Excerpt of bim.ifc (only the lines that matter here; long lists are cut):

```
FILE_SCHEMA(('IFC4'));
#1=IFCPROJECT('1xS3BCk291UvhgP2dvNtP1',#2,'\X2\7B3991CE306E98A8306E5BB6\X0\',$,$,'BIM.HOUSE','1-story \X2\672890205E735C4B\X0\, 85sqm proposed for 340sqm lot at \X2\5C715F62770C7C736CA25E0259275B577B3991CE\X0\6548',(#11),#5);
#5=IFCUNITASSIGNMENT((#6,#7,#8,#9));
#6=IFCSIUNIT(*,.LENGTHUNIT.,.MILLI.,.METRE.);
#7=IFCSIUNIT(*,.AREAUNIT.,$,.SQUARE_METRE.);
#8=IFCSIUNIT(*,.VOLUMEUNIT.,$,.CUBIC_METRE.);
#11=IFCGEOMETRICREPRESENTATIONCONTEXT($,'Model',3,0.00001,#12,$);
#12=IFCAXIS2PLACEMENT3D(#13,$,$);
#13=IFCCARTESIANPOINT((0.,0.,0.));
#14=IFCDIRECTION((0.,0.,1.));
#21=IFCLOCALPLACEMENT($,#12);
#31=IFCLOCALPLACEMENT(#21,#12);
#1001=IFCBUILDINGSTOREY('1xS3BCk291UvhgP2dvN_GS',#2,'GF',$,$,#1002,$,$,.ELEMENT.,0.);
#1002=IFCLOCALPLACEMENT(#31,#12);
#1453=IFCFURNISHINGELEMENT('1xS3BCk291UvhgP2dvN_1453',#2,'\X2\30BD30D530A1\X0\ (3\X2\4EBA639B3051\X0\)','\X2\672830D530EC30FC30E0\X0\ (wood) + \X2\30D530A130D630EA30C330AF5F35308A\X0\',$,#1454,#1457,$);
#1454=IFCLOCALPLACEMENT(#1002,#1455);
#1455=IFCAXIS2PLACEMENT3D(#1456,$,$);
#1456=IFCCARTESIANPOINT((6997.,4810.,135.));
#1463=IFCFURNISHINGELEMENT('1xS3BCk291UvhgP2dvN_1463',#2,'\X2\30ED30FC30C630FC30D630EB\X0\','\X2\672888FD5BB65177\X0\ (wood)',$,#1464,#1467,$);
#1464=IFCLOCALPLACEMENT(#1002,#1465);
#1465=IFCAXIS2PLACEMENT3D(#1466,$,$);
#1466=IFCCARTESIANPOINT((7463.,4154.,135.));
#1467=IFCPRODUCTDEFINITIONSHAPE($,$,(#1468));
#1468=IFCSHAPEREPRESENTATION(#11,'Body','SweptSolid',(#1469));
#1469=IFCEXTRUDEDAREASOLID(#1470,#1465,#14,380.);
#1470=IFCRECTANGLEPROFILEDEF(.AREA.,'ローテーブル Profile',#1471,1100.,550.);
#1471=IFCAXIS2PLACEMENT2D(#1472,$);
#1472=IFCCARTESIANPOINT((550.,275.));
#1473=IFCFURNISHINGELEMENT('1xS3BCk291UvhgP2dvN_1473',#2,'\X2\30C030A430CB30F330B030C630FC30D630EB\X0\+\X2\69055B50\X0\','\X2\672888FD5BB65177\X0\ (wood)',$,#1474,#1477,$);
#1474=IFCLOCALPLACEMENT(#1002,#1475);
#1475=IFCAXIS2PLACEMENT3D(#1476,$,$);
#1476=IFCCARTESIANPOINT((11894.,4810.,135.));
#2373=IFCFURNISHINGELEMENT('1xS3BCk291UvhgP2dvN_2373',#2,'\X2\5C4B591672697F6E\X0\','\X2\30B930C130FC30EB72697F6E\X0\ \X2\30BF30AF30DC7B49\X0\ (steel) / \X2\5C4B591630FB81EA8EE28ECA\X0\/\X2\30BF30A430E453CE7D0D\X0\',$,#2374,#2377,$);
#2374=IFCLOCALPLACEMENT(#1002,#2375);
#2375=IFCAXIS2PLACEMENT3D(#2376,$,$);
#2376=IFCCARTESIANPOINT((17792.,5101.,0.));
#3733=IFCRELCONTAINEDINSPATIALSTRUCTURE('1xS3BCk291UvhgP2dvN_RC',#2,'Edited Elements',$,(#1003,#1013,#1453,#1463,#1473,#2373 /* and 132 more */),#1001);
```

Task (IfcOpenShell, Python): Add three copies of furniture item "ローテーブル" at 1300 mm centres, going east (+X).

```python
import numpy as np
import ifcopenshell
import ifcopenshell.api.geometry
import ifcopenshell.api.root
import ifcopenshell.util.element
import ifcopenshell.util.placement

model = ifcopenshell.open("bim.ifc")


def reuse_history(source, copy):
    """copy_class also copies each property set's owner history, people and application; keep the originals."""
    for rel in copy.IsDefinedBy:
        if rel.is_a("IfcRelDefinesByProperties") and (history := rel.RelatingPropertyDefinition.OwnerHistory):
            rel.RelatingPropertyDefinition.OwnerHistory = source.OwnerHistory
            ifcopenshell.util.element.remove_deep2(model, history)


source = model.by_guid("1xS3BCk291UvhgP2dvN_1463")
base = ifcopenshell.util.placement.get_local_placement(source.ObjectPlacement)
step = np.array([1.0, 0.0, 0.0]) * 1300.0

for i in range(1, 4):
    copy = ifcopenshell.api.root.copy_class(model, product=source)
    copy.Representation = ifcopenshell.util.element.copy_deep(
        model, source.Representation, exclude=["IfcGeometricRepresentationContext", "IfcRepresentationMap"]
    )
    reuse_history(source, copy)
    matrix = base.copy()
    matrix[:3, 3] += i * step
    print("added at", matrix[:3, 3].round(3) + 0.0)
    ifcopenshell.api.geometry.edit_object_placement(model, product=copy, matrix=matrix, is_si=False)

model.write("bim_updated.ifc")
```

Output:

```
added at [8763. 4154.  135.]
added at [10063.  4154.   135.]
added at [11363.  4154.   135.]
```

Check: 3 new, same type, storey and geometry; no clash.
